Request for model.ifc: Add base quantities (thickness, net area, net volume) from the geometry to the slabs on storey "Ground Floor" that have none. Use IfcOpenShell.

First a look at what the model holds.

```python
import ifcopenshell
import ifcopenshell.util.element
import ifcopenshell.util.unit

model = ifcopenshell.open("model.ifc")
print(model.schema)
for unit_type in ("LENGTHUNIT", "AREAUNIT", "VOLUMEUNIT"):
    print(unit_type, ifcopenshell.util.unit.calculate_unit_scale(model, unit_type))
storey = next(s for s in model.by_type("IfcBuildingStorey") if s.Name == "Ground Floor")
slabs = [e for e in ifcopenshell.util.element.get_decomposition(storey) if e.is_a("IfcSlab")]
for e in sorted(slabs, key=lambda e: e.id()):
    print(e.id(), e.is_a(), e.Name, list(ifcopenshell.util.element.get_psets(e, qtos_only=True)), sep=" | ")
```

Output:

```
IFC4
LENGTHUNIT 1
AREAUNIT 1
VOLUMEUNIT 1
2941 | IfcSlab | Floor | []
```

```python
import ifcopenshell
import ifcopenshell.api.pset
import ifcopenshell.geom
import ifcopenshell.util.element
import ifcopenshell.util.shape
import ifcopenshell.util.unit

model = ifcopenshell.open("model.ifc")
unit_scale = ifcopenshell.util.unit.calculate_unit_scale(model)
area_scale = ifcopenshell.util.unit.calculate_unit_scale(model, "AREAUNIT")
volume_scale = ifcopenshell.util.unit.calculate_unit_scale(model, "VOLUMEUNIT")
settings = ifcopenshell.geom.settings()

storey = next(s for s in model.by_type("IfcBuildingStorey") if s.Name == "Ground Floor")
slabs = [e for e in ifcopenshell.util.element.get_decomposition(storey) if e.is_a("IfcSlab")]

for e in sorted(slabs, key=lambda e: e.id()):
    if ifcopenshell.util.element.get_psets(e, qtos_only=True, should_inherit=False):
        continue
    # Geometry comes back in metres, in the element's own axes.
    shape = ifcopenshell.geom.create_shape(settings, e)
    values = {
        "Width": ifcopenshell.util.shape.get_z(shape.geometry) / unit_scale,
        "NetArea": ifcopenshell.util.shape.get_footprint_area(shape.geometry) / area_scale,
        "NetVolume": ifcopenshell.util.shape.get_volume(shape.geometry) / volume_scale,
    }
    qto = ifcopenshell.api.pset.add_qto(model, product=e, name="Qto_SlabBaseQuantities")
    ifcopenshell.api.pset.edit_qto(model, qto=qto, properties=values)
    print(e.id(), {k: round(v, 3) for k, v in values.items()})

model.write("model_rev.ifc")
```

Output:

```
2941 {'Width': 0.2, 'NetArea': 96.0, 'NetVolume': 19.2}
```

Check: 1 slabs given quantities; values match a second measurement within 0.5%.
